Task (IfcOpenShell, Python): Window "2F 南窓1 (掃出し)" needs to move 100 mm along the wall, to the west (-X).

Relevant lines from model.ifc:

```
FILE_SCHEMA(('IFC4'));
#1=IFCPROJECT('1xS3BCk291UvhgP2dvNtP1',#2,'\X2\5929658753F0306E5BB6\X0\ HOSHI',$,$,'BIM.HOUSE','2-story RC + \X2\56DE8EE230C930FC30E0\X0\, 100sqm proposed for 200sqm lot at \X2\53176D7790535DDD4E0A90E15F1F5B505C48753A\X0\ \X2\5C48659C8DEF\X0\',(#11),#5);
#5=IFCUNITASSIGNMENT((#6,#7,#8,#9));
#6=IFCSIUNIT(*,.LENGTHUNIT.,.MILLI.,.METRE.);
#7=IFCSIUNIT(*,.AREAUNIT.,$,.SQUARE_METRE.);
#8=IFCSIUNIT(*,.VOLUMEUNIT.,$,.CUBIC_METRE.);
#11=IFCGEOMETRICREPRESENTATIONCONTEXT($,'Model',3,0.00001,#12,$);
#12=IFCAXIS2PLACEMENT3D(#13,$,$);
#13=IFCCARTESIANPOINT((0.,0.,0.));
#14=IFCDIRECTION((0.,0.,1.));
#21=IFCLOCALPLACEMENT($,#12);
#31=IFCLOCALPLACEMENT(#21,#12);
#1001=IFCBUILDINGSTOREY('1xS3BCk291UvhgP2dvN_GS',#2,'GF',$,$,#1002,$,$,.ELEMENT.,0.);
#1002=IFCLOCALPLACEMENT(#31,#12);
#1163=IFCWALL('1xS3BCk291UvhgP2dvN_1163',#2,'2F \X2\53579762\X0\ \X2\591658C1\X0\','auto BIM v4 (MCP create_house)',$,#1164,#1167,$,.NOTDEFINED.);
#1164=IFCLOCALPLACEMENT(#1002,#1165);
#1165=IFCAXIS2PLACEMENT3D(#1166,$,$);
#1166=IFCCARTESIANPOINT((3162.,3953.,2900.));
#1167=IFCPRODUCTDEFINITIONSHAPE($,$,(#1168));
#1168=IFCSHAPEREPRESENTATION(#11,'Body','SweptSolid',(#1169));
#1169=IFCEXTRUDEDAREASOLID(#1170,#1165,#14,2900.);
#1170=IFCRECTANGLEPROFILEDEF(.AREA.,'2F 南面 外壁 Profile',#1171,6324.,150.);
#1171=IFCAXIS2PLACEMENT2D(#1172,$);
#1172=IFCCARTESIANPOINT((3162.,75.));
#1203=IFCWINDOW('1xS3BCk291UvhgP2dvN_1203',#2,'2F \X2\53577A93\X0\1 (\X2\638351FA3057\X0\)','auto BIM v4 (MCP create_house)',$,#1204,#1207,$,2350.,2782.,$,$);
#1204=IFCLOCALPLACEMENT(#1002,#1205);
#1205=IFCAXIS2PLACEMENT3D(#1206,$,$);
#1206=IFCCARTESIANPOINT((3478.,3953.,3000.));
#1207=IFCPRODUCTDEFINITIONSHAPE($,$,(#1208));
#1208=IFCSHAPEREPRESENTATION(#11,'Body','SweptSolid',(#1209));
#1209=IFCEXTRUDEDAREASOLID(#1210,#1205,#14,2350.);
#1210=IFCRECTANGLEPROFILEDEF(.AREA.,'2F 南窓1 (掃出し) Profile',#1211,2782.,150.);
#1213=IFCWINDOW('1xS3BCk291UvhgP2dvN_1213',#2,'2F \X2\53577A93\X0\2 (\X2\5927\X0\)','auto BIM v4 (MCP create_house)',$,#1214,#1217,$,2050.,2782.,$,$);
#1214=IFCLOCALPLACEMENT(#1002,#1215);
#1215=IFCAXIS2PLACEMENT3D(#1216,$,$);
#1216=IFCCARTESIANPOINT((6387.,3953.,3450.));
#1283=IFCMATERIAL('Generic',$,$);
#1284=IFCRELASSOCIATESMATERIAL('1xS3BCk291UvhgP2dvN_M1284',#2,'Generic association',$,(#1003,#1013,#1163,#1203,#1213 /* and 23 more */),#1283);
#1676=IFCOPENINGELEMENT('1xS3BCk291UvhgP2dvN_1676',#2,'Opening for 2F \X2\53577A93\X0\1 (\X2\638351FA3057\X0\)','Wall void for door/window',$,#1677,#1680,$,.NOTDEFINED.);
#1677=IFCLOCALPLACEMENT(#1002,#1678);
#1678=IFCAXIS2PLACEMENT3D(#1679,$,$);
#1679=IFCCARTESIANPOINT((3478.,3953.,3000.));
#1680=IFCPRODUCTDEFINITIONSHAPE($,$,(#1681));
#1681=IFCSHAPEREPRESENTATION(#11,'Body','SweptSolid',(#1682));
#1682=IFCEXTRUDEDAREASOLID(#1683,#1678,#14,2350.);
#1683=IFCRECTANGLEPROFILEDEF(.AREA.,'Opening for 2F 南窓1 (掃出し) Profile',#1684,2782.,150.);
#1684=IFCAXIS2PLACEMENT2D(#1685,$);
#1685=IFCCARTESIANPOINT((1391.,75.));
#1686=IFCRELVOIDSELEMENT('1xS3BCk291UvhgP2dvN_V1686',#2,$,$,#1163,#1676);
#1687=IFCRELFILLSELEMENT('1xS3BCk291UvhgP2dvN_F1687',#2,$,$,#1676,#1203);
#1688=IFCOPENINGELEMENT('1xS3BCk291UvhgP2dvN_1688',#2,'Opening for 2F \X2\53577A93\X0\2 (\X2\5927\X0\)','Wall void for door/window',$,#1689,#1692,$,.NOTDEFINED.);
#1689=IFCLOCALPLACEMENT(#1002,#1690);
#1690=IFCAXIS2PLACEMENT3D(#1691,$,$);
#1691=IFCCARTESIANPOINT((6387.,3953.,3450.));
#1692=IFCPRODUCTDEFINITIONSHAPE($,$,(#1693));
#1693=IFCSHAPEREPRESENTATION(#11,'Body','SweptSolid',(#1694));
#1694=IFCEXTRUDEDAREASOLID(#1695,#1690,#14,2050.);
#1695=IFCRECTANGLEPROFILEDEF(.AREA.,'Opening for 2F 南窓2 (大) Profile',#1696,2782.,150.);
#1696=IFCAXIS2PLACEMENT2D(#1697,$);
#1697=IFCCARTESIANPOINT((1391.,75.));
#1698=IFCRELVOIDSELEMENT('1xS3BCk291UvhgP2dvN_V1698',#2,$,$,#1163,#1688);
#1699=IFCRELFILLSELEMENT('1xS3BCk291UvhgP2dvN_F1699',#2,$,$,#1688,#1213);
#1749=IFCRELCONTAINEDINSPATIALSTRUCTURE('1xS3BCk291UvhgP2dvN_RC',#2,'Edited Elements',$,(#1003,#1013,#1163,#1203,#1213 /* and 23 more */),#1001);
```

```python
import ifcopenshell
import ifcopenshell.api.geometry
import ifcopenshell.util.placement

model = ifcopenshell.open("model.ifc")

window = model.by_guid("1xS3BCk291UvhgP2dvN_1203")
opening = window.FillsVoids[0].RelatingOpeningElement
wall = opening.VoidsElements[0].RelatingBuildingElement

wall_matrix = ifcopenshell.util.placement.get_local_placement(wall.ObjectPlacement)
shift = wall_matrix[:3, 0] * -100.0
before = ifcopenshell.util.placement.get_local_placement(window.ObjectPlacement)[:3, 3].copy()

# The window is not placed relative to its opening, so move both.
for product in (opening, window):
    matrix = ifcopenshell.util.placement.get_local_placement(product.ObjectPlacement)
    matrix[:3, 3] += shift
    ifcopenshell.api.geometry.edit_object_placement(model, product=product, matrix=matrix, is_si=False)

after = ifcopenshell.util.placement.get_local_placement(window.ObjectPlacement)[:3, 3]
print("window moved by", (after - before).round(3) + 0.0)

model.write("model-out.ifc")
```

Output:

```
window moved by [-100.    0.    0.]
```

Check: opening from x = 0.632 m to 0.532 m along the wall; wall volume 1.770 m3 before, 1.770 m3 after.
